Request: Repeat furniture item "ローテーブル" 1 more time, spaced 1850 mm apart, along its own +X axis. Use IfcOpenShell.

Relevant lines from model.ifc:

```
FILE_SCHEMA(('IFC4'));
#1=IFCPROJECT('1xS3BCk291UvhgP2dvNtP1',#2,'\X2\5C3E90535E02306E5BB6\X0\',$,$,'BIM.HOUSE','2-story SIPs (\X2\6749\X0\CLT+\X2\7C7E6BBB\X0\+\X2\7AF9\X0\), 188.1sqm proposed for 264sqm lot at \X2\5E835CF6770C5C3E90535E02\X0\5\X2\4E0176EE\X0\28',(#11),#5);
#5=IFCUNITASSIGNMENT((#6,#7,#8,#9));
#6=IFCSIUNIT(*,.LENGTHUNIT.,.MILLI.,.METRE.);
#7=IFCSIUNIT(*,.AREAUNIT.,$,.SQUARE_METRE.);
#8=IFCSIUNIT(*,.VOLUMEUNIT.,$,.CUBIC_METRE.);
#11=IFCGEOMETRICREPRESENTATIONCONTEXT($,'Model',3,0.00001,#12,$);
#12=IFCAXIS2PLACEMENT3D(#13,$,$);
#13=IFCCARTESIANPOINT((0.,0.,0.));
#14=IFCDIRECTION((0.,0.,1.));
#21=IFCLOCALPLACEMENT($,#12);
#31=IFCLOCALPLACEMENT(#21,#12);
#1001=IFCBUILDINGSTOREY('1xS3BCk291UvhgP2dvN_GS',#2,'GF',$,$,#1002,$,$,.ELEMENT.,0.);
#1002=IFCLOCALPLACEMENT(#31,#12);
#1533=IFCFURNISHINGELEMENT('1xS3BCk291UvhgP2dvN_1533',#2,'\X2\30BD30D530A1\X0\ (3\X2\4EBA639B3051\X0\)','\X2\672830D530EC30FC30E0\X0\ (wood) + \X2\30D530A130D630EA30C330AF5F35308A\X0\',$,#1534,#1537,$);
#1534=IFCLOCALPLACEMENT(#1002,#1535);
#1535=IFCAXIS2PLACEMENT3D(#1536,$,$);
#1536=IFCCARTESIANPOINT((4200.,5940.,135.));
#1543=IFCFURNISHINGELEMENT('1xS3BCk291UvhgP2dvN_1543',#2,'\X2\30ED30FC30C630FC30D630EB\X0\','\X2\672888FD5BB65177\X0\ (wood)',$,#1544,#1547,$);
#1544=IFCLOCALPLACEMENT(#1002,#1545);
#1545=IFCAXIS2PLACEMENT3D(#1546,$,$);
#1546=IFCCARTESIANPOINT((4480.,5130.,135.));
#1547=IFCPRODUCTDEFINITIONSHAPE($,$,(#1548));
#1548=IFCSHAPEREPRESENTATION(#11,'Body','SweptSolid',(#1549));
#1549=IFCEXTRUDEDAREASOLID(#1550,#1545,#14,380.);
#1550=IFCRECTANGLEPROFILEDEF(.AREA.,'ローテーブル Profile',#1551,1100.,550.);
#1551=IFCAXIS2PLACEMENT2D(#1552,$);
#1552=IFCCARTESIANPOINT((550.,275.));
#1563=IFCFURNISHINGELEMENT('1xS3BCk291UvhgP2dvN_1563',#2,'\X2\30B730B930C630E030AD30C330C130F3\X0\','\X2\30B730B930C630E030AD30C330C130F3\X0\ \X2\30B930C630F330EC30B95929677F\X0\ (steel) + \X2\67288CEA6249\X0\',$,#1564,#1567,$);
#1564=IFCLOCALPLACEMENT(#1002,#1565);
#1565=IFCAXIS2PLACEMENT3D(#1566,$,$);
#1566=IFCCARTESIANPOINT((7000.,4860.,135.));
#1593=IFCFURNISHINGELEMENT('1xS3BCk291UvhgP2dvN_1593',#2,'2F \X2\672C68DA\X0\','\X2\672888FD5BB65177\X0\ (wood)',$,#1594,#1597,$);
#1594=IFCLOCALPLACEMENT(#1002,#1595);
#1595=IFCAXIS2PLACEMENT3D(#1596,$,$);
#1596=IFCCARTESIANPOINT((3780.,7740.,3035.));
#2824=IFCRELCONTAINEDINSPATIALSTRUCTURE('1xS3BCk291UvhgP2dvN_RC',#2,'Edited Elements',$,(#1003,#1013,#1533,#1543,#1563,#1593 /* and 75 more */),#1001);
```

```python
import ifcopenshell
import ifcopenshell.api.geometry
import ifcopenshell.api.root
import ifcopenshell.util.element
import ifcopenshell.util.placement
import ifcopenshell.util.unit

model = ifcopenshell.open("model.ifc")
unit_scale = ifcopenshell.util.unit.calculate_unit_scale(model)


def reuse_history(source, copy):
    """copy_class also copies each property set's owner history, people and application; keep the originals."""
    for rel in copy.IsDefinedBy:
        if rel.is_a("IfcRelDefinesByProperties") and (history := rel.RelatingPropertyDefinition.OwnerHistory):
            rel.RelatingPropertyDefinition.OwnerHistory = source.OwnerHistory
            ifcopenshell.util.element.remove_deep2(model, history)


source = model.by_guid("1xS3BCk291UvhgP2dvN_1543")
base = ifcopenshell.util.placement.get_local_placement(source.ObjectPlacement)
step = base[:3, 0] * 1.85 / unit_scale

for i in range(1, 2):
    copy = ifcopenshell.api.root.copy_class(model, product=source)
    copy.Representation = ifcopenshell.util.element.copy_deep(
        model, source.Representation, exclude=["IfcGeometricRepresentationContext", "IfcRepresentationMap"]
    )
    reuse_history(source, copy)
    matrix = base.copy()
    matrix[:3, 3] += i * step
    print("added at", matrix[:3, 3].round(3) + 0.0)
    ifcopenshell.api.geometry.edit_object_placement(model, product=copy, matrix=matrix, is_si=False)

model.write("model_updated.ifc")
```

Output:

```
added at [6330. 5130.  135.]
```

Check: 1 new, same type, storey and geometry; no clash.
